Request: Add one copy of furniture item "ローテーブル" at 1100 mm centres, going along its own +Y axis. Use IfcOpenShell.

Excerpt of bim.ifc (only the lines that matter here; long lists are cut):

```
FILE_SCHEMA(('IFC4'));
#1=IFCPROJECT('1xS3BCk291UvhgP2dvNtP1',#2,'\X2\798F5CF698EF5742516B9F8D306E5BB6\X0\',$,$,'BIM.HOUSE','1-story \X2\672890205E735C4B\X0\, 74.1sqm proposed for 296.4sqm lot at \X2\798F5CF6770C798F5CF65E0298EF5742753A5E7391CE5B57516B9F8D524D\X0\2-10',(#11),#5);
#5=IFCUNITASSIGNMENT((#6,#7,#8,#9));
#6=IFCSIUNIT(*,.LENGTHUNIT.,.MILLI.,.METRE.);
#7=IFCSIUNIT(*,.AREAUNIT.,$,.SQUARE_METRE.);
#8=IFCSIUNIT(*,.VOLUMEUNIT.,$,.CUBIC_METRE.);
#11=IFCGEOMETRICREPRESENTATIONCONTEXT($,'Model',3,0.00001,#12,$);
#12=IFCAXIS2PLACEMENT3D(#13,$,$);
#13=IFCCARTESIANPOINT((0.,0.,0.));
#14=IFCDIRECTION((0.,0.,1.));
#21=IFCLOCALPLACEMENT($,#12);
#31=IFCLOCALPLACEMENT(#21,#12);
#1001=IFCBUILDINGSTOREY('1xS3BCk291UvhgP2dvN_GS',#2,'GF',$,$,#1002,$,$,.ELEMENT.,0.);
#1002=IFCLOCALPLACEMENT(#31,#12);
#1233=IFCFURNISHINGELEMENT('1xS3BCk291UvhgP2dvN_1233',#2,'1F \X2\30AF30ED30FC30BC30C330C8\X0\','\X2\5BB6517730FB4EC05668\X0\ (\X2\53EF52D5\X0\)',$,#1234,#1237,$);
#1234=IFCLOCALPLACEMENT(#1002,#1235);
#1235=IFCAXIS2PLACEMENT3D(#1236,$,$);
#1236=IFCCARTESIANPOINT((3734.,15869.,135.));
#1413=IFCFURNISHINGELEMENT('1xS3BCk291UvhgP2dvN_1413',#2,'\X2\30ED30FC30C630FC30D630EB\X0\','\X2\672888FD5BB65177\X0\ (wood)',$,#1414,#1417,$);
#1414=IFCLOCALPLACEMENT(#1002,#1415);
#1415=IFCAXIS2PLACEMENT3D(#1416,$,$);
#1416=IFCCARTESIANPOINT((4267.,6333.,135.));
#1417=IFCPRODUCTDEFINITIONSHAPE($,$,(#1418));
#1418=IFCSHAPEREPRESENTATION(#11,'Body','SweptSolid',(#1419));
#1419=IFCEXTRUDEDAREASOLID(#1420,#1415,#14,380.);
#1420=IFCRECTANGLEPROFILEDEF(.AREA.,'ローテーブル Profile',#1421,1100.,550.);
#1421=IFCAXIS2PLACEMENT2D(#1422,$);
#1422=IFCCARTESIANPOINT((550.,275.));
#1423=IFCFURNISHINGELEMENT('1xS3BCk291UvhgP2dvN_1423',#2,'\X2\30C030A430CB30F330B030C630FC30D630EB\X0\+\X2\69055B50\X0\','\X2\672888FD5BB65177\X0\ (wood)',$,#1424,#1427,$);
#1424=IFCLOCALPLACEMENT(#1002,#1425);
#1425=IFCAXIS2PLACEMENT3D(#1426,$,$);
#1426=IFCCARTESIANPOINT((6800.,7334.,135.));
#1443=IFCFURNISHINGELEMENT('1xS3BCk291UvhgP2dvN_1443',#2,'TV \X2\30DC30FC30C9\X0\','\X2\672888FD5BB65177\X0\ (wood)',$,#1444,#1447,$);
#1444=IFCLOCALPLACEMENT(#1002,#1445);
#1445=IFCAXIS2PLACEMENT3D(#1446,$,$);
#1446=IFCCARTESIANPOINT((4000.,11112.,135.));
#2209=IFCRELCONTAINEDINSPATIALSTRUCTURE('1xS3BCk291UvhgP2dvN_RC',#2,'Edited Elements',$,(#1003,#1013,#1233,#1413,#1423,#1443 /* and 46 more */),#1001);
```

```python
import ifcopenshell
import ifcopenshell.api.geometry
import ifcopenshell.api.root
import ifcopenshell.util.element
import ifcopenshell.util.placement
import ifcopenshell.util.unit

model = ifcopenshell.open("bim.ifc")
unit_scale = ifcopenshell.util.unit.calculate_unit_scale(model)


def reuse_history(source, copy):
    """copy_class also copies each property set's owner history, people and application; keep the originals."""
    for rel in copy.IsDefinedBy:
        if rel.is_a("IfcRelDefinesByProperties") and (history := rel.RelatingPropertyDefinition.OwnerHistory):
            rel.RelatingPropertyDefinition.OwnerHistory = source.OwnerHistory
            ifcopenshell.util.element.remove_deep2(model, history)


source = model.by_id(1413)
base = ifcopenshell.util.placement.get_local_placement(source.ObjectPlacement)
step = base[:3, 1] * 1.1 / unit_scale

for i in range(1, 2):
    copy = ifcopenshell.api.root.copy_class(model, product=source)
    copy.Representation = ifcopenshell.util.element.copy_deep(
        model, source.Representation, exclude=["IfcGeometricRepresentationContext", "IfcRepresentationMap"]
    )
    reuse_history(source, copy)
    matrix = base.copy()
    matrix[:3, 3] += i * step
    print("added at", matrix[:3, 3].round(3) + 0.0)
    ifcopenshell.api.geometry.edit_object_placement(model, product=copy, matrix=matrix, is_si=False)

model.write("bim-out.ifc")
```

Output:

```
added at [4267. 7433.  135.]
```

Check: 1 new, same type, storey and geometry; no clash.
